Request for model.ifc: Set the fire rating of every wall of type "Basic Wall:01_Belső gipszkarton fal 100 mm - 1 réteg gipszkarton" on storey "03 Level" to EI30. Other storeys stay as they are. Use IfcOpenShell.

First a look at what the model holds.

```python
import ifcopenshell
import ifcopenshell.util.element

model = ifcopenshell.open("model.ifc")
print(model.schema)
storey = next(s for s in model.by_type("IfcBuildingStorey") if s.Name == "03 Level")
walls = [e for e in ifcopenshell.util.element.get_decomposition(storey) if e.is_a("IfcWall")]
seen = {}
for e in walls:
    element_type = ifcopenshell.util.element.get_type(e)
    key = (element_type.Name if element_type != e and element_type else None, ifcopenshell.util.element.get_pset(e, "Pset_WallCommon", "FireRating"))
    seen[key] = seen.get(key, 0) + 1
for (name, value), count in sorted(seen.items(), key=str):
    print(count, "x", name, "|", value)
```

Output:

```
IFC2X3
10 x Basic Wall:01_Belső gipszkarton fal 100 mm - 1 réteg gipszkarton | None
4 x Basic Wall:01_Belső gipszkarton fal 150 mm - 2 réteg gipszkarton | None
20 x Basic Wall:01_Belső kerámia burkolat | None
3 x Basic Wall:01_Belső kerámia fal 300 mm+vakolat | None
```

```python
import ifcopenshell
import ifcopenshell.api.pset
import ifcopenshell.util.element

model = ifcopenshell.open("model.ifc")

storey = next(s for s in model.by_type("IfcBuildingStorey") if s.Name == "03 Level")
walls = [e for e in ifcopenshell.util.element.get_decomposition(storey) if e.is_a("IfcWall")]

count = 0
for e in walls:
    element_type = ifcopenshell.util.element.get_type(e)
    if element_type in (None, e) or element_type.Name != "Basic Wall:01_Belső gipszkarton fal 100 mm - 1 réteg gipszkarton":
        continue
    # add_pset returns the element's existing set when there is one.
    pset = ifcopenshell.api.pset.add_pset(model, product=e, name="Pset_WallCommon")
    ifcopenshell.api.pset.edit_pset(model, pset=pset, properties={"FireRating": "EI30"})
    count += 1

print(count, "walls updated")

model.write("model_edited.ifc")
```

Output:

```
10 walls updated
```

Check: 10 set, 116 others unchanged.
